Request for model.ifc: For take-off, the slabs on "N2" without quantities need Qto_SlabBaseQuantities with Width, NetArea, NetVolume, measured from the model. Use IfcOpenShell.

First a look at what the model holds.

```python
import ifcopenshell
import ifcopenshell.util.element
import ifcopenshell.util.unit

model = ifcopenshell.open("model.ifc")
print(model.schema)
for unit_type in ("LENGTHUNIT", "AREAUNIT", "VOLUMEUNIT"):
    print(unit_type, ifcopenshell.util.unit.calculate_unit_scale(model, unit_type))
storey = next(s for s in model.by_type("IfcBuildingStorey") if s.Name == "N2")
slabs = [e for e in ifcopenshell.util.element.get_decomposition(storey) if e.is_a("IfcSlab")]
for e in sorted(slabs, key=lambda e: e.id()):
    print(e.id(), e.is_a(), e.Name, list(ifcopenshell.util.element.get_psets(e, qtos_only=True)), sep=" | ")
```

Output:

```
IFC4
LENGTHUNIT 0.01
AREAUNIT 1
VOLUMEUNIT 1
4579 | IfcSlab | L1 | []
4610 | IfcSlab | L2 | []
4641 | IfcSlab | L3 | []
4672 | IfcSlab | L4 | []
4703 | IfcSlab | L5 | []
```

```python
import ifcopenshell
import ifcopenshell.api.pset
import ifcopenshell.geom
import ifcopenshell.util.element
import ifcopenshell.util.shape
import ifcopenshell.util.unit

model = ifcopenshell.open("model.ifc")
unit_scale = ifcopenshell.util.unit.calculate_unit_scale(model)
area_scale = ifcopenshell.util.unit.calculate_unit_scale(model, "AREAUNIT")
volume_scale = ifcopenshell.util.unit.calculate_unit_scale(model, "VOLUMEUNIT")
settings = ifcopenshell.geom.settings()

storey = next(s for s in model.by_type("IfcBuildingStorey") if s.Name == "N2")
slabs = [e for e in ifcopenshell.util.element.get_decomposition(storey) if e.is_a("IfcSlab")]

for e in sorted(slabs, key=lambda e: e.id()):
    if ifcopenshell.util.element.get_psets(e, qtos_only=True, should_inherit=False):
        continue
    # Geometry comes back in metres, in the element's own axes.
    shape = ifcopenshell.geom.create_shape(settings, e)
    values = {
        "Width": ifcopenshell.util.shape.get_z(shape.geometry) / unit_scale,
        "NetArea": ifcopenshell.util.shape.get_footprint_area(shape.geometry) / area_scale,
        "NetVolume": ifcopenshell.util.shape.get_volume(shape.geometry) / volume_scale,
    }
    qto = ifcopenshell.api.pset.add_qto(model, product=e, name="Qto_SlabBaseQuantities")
    ifcopenshell.api.pset.edit_qto(model, qto=qto, properties=values)
    print(e.id(), {k: round(v, 3) for k, v in values.items()})

model.write("model_edited.ifc")
```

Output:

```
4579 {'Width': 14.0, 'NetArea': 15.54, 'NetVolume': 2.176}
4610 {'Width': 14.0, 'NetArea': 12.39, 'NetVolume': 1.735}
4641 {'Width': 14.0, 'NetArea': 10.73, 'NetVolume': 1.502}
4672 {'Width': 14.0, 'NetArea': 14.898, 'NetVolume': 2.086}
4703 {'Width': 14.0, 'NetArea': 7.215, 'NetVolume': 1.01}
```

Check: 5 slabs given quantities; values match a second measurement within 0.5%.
